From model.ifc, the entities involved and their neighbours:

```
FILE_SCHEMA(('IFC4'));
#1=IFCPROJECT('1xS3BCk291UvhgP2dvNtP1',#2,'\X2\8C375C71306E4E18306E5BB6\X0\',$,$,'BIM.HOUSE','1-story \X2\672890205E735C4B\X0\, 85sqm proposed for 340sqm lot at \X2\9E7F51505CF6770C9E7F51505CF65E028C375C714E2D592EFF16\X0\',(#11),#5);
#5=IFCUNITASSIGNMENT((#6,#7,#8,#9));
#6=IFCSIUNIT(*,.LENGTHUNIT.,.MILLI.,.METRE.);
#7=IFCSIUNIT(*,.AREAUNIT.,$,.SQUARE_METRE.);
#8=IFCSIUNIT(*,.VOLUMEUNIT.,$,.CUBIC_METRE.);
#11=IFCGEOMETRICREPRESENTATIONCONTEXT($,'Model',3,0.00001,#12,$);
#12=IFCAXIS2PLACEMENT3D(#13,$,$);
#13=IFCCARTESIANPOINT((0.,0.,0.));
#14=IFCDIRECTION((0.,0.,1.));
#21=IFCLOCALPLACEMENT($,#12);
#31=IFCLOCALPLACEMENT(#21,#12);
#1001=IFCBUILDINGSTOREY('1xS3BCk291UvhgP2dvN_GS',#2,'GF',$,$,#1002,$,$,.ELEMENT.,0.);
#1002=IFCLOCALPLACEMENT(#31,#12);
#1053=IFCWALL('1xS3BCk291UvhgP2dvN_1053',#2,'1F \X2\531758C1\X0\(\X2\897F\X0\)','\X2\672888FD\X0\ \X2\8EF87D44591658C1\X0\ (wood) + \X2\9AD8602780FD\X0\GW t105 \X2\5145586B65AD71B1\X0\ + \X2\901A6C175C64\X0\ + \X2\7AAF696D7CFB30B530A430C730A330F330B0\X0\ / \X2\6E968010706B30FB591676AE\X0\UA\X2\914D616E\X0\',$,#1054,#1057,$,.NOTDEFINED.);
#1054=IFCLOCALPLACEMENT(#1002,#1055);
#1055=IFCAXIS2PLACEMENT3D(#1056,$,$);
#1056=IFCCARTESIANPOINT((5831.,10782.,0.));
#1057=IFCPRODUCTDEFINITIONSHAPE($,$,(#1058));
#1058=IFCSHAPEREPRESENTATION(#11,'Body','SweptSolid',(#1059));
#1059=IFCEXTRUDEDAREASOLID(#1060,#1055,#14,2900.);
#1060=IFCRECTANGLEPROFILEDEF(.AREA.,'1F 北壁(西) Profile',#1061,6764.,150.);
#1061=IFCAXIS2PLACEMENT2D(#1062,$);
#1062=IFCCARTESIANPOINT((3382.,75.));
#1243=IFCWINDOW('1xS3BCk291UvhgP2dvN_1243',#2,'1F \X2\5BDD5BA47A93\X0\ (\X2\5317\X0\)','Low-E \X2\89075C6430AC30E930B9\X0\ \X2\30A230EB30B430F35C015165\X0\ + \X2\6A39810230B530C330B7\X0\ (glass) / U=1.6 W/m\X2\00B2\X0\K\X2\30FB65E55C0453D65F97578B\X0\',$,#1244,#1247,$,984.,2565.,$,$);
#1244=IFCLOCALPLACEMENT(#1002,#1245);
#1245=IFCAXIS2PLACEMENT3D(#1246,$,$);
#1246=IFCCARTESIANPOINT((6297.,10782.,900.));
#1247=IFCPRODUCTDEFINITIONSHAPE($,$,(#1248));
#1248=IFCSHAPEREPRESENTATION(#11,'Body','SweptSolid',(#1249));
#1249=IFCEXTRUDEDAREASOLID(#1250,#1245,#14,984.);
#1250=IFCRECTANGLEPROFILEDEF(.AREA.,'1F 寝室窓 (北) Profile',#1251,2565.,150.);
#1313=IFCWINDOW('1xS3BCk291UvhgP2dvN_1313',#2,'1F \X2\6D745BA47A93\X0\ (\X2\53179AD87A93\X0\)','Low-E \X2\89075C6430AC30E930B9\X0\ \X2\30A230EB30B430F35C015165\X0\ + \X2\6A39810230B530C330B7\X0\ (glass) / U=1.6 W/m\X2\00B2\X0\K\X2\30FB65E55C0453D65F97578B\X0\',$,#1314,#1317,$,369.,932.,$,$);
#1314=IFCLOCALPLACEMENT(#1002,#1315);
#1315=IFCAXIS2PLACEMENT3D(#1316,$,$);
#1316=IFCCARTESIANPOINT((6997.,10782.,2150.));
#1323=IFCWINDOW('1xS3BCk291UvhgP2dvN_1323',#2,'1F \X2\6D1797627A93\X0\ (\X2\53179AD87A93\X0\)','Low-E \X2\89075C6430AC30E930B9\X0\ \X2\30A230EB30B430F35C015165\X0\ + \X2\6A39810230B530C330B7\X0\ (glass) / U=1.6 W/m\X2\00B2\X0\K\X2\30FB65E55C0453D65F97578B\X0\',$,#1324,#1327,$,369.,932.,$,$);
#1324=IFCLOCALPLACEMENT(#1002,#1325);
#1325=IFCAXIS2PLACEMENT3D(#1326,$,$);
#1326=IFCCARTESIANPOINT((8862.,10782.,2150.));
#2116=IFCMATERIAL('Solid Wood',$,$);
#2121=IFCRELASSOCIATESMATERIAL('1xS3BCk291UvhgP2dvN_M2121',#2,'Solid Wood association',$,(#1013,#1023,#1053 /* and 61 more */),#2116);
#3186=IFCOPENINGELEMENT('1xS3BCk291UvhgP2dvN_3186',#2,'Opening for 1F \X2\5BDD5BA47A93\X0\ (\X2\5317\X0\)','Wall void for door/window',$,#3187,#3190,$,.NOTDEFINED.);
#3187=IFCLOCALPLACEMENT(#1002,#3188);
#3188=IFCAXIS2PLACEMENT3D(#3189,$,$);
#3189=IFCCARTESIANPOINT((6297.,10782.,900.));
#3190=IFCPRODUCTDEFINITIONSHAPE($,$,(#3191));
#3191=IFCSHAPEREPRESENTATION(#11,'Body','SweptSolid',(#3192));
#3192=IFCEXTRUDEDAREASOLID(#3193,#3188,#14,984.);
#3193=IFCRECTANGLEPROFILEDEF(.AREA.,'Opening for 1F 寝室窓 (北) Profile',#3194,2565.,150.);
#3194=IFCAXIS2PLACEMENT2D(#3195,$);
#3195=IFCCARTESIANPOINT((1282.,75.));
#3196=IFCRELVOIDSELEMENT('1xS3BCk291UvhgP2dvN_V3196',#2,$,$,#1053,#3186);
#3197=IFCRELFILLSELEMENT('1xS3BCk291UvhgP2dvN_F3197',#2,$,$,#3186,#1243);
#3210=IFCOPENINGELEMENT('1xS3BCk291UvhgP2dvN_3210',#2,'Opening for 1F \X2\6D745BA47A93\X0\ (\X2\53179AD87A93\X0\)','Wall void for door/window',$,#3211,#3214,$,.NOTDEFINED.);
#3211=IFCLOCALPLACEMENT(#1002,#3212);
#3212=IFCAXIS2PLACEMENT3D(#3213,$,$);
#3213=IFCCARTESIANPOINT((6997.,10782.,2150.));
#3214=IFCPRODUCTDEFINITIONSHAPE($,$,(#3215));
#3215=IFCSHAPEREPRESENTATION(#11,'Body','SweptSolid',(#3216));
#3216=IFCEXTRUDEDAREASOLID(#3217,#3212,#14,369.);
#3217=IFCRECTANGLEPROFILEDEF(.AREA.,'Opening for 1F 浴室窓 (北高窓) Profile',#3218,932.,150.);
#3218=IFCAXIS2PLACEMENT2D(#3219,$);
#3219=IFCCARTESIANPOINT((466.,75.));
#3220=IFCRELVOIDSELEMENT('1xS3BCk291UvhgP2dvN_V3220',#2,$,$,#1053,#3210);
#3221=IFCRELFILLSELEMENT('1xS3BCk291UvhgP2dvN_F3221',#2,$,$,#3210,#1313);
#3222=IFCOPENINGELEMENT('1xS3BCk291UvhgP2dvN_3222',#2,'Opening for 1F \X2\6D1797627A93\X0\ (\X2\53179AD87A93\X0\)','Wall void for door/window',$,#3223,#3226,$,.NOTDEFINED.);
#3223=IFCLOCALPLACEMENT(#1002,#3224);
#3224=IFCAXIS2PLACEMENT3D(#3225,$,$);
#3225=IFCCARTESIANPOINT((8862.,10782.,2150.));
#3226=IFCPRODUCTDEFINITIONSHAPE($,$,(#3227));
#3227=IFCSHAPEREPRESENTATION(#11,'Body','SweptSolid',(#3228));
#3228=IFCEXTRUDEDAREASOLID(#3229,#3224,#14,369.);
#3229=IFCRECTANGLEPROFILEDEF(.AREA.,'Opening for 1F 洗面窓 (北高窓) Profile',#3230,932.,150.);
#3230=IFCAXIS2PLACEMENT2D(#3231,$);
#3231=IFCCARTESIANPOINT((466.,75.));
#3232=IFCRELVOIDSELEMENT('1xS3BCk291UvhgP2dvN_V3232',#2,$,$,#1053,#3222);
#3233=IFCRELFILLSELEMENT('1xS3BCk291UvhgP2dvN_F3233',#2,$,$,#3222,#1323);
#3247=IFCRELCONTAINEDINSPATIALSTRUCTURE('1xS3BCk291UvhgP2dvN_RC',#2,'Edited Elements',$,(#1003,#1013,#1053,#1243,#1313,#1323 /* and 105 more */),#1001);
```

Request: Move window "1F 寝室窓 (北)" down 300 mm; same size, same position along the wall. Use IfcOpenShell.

```python
import numpy as np
import ifcopenshell
import ifcopenshell.api.geometry
import ifcopenshell.util.placement
import ifcopenshell.util.unit

model = ifcopenshell.open("model.ifc")
unit_scale = ifcopenshell.util.unit.calculate_unit_scale(model)

window = model.by_guid("1xS3BCk291UvhgP2dvN_1243")
opening = window.FillsVoids[0].RelatingOpeningElement
dz = -300.0

shift = np.array([0.0, 0.0, dz])
# The window is not placed relative to its opening, so move both.
for product in (opening, window):
    matrix = ifcopenshell.util.placement.get_local_placement(product.ObjectPlacement)
    matrix[:3, 3] += shift
    ifcopenshell.api.geometry.edit_object_placement(model, product=product, matrix=matrix, is_si=False)

print(f"moved by {dz * unit_scale:+.3f} m")

model.write("model-out.ifc")
```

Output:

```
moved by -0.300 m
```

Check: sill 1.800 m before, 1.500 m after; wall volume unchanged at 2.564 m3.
